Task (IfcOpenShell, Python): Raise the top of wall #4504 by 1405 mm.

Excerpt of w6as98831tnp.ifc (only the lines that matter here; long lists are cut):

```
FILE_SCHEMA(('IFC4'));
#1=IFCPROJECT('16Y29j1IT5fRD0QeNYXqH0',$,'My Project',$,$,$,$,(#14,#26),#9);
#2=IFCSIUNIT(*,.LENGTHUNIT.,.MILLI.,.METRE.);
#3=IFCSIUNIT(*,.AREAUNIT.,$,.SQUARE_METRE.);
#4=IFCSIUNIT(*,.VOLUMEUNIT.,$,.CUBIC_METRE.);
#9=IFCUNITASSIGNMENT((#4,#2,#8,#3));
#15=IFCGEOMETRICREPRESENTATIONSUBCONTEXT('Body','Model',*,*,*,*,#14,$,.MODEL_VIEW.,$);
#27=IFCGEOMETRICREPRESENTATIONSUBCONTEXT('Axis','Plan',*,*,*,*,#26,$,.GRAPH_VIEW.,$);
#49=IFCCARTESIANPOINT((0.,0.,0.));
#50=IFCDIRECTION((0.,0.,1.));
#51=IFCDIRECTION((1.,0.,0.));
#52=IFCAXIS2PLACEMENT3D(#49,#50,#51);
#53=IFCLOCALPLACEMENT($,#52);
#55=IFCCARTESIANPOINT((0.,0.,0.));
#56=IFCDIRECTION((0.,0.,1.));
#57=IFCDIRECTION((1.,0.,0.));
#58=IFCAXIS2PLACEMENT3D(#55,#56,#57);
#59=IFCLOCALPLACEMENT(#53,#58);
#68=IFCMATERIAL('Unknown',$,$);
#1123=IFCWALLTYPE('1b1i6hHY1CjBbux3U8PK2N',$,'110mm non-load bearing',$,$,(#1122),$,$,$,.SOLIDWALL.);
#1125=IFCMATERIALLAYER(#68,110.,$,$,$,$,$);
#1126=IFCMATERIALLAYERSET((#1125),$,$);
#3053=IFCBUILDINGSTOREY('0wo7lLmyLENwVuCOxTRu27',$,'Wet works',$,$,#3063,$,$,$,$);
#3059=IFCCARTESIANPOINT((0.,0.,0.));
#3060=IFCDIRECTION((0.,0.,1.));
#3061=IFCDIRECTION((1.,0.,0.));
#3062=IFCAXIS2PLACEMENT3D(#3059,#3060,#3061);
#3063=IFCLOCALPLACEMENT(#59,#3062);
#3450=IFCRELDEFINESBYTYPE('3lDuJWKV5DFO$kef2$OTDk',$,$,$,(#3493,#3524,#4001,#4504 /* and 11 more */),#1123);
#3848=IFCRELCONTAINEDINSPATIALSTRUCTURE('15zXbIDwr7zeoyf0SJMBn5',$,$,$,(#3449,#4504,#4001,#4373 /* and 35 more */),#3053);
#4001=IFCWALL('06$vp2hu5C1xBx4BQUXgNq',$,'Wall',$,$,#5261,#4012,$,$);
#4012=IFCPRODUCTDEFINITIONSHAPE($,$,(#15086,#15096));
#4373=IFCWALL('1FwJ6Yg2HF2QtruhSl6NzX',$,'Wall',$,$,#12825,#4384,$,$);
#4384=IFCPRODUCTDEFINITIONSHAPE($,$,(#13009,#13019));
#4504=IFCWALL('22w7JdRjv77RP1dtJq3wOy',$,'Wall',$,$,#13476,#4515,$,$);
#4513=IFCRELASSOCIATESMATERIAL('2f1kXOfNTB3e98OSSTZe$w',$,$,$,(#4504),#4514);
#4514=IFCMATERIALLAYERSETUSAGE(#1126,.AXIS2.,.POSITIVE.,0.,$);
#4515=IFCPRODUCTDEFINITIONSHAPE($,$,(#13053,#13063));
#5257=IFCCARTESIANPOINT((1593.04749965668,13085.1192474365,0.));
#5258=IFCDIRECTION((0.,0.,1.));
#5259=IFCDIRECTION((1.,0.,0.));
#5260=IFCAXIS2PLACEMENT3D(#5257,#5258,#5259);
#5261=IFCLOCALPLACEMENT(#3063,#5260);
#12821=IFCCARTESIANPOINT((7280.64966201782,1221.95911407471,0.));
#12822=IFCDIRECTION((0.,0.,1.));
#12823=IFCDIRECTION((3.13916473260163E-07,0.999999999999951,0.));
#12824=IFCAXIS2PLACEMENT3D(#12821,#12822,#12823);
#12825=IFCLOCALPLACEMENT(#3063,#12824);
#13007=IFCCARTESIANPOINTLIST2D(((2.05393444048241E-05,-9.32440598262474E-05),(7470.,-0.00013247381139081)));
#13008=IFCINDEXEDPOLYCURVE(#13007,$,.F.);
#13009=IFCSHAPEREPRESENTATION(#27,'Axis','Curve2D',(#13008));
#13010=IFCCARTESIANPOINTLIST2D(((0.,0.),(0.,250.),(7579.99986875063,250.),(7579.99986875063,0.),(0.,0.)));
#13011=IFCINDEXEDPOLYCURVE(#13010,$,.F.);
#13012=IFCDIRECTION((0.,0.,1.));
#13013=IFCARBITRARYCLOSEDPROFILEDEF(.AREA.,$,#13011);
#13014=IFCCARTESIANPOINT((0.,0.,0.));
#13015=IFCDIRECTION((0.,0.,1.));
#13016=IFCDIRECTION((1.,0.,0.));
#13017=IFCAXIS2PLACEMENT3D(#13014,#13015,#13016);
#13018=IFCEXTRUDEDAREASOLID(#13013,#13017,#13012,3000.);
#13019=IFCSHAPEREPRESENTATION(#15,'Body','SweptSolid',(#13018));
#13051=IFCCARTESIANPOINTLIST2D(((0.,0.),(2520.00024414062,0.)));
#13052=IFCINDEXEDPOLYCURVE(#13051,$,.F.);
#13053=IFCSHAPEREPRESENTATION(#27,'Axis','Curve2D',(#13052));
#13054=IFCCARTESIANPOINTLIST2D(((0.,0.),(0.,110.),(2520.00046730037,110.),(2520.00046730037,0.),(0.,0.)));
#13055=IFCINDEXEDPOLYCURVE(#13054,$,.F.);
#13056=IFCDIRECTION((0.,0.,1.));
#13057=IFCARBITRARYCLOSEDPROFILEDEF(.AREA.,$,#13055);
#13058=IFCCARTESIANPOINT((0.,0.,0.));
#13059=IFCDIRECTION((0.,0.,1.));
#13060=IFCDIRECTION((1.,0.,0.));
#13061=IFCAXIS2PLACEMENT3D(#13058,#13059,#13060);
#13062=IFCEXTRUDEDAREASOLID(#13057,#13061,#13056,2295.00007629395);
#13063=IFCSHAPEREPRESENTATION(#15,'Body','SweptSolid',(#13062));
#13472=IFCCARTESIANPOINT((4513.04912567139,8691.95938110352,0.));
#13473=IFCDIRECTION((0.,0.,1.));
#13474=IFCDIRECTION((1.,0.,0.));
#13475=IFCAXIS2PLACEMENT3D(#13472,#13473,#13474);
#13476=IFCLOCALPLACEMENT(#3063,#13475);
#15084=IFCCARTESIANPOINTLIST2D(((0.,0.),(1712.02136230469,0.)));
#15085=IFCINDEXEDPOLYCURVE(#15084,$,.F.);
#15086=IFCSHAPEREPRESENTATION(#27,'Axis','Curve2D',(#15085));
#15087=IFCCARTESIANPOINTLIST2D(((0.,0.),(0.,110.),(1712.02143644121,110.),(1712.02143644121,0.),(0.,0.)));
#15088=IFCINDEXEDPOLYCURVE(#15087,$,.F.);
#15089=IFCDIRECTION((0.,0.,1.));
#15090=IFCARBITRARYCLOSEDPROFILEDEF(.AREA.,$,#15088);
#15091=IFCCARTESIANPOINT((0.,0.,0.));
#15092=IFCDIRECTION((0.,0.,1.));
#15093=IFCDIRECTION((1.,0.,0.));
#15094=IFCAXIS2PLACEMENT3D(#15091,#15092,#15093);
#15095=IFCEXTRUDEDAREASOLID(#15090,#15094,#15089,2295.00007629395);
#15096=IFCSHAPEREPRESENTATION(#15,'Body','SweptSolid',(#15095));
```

```python
import ifcopenshell
import ifcopenshell.geom
import ifcopenshell.util.representation
import ifcopenshell.util.shape
import ifcopenshell.util.unit

model = ifcopenshell.open("w6as98831tnp.ifc")
unit_scale = ifcopenshell.util.unit.calculate_unit_scale(model)
settings = ifcopenshell.geom.settings()


def volume(element):
    """Net volume in cubic metres, openings subtracted."""
    shape = ifcopenshell.geom.create_shape(settings, element)
    return ifcopenshell.util.shape.get_volume(shape.geometry)


wall = model.by_guid("22w7JdRjv77RP1dtJq3wOy")
before = volume(wall)

body = ifcopenshell.util.representation.get_representation(wall, "Model", "Body")
solid = body.Items[0]
old_height = solid.Depth
solid.Depth += 1.405 / unit_scale
after = volume(wall)

print(f"height {old_height:g} -> {solid.Depth:g}, volume {before:.3f} -> {after:.3f} m3")

model.write("w6as98831tnp_updated.ifc")
```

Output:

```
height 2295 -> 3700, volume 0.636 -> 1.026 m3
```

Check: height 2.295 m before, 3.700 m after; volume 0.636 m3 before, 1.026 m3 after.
